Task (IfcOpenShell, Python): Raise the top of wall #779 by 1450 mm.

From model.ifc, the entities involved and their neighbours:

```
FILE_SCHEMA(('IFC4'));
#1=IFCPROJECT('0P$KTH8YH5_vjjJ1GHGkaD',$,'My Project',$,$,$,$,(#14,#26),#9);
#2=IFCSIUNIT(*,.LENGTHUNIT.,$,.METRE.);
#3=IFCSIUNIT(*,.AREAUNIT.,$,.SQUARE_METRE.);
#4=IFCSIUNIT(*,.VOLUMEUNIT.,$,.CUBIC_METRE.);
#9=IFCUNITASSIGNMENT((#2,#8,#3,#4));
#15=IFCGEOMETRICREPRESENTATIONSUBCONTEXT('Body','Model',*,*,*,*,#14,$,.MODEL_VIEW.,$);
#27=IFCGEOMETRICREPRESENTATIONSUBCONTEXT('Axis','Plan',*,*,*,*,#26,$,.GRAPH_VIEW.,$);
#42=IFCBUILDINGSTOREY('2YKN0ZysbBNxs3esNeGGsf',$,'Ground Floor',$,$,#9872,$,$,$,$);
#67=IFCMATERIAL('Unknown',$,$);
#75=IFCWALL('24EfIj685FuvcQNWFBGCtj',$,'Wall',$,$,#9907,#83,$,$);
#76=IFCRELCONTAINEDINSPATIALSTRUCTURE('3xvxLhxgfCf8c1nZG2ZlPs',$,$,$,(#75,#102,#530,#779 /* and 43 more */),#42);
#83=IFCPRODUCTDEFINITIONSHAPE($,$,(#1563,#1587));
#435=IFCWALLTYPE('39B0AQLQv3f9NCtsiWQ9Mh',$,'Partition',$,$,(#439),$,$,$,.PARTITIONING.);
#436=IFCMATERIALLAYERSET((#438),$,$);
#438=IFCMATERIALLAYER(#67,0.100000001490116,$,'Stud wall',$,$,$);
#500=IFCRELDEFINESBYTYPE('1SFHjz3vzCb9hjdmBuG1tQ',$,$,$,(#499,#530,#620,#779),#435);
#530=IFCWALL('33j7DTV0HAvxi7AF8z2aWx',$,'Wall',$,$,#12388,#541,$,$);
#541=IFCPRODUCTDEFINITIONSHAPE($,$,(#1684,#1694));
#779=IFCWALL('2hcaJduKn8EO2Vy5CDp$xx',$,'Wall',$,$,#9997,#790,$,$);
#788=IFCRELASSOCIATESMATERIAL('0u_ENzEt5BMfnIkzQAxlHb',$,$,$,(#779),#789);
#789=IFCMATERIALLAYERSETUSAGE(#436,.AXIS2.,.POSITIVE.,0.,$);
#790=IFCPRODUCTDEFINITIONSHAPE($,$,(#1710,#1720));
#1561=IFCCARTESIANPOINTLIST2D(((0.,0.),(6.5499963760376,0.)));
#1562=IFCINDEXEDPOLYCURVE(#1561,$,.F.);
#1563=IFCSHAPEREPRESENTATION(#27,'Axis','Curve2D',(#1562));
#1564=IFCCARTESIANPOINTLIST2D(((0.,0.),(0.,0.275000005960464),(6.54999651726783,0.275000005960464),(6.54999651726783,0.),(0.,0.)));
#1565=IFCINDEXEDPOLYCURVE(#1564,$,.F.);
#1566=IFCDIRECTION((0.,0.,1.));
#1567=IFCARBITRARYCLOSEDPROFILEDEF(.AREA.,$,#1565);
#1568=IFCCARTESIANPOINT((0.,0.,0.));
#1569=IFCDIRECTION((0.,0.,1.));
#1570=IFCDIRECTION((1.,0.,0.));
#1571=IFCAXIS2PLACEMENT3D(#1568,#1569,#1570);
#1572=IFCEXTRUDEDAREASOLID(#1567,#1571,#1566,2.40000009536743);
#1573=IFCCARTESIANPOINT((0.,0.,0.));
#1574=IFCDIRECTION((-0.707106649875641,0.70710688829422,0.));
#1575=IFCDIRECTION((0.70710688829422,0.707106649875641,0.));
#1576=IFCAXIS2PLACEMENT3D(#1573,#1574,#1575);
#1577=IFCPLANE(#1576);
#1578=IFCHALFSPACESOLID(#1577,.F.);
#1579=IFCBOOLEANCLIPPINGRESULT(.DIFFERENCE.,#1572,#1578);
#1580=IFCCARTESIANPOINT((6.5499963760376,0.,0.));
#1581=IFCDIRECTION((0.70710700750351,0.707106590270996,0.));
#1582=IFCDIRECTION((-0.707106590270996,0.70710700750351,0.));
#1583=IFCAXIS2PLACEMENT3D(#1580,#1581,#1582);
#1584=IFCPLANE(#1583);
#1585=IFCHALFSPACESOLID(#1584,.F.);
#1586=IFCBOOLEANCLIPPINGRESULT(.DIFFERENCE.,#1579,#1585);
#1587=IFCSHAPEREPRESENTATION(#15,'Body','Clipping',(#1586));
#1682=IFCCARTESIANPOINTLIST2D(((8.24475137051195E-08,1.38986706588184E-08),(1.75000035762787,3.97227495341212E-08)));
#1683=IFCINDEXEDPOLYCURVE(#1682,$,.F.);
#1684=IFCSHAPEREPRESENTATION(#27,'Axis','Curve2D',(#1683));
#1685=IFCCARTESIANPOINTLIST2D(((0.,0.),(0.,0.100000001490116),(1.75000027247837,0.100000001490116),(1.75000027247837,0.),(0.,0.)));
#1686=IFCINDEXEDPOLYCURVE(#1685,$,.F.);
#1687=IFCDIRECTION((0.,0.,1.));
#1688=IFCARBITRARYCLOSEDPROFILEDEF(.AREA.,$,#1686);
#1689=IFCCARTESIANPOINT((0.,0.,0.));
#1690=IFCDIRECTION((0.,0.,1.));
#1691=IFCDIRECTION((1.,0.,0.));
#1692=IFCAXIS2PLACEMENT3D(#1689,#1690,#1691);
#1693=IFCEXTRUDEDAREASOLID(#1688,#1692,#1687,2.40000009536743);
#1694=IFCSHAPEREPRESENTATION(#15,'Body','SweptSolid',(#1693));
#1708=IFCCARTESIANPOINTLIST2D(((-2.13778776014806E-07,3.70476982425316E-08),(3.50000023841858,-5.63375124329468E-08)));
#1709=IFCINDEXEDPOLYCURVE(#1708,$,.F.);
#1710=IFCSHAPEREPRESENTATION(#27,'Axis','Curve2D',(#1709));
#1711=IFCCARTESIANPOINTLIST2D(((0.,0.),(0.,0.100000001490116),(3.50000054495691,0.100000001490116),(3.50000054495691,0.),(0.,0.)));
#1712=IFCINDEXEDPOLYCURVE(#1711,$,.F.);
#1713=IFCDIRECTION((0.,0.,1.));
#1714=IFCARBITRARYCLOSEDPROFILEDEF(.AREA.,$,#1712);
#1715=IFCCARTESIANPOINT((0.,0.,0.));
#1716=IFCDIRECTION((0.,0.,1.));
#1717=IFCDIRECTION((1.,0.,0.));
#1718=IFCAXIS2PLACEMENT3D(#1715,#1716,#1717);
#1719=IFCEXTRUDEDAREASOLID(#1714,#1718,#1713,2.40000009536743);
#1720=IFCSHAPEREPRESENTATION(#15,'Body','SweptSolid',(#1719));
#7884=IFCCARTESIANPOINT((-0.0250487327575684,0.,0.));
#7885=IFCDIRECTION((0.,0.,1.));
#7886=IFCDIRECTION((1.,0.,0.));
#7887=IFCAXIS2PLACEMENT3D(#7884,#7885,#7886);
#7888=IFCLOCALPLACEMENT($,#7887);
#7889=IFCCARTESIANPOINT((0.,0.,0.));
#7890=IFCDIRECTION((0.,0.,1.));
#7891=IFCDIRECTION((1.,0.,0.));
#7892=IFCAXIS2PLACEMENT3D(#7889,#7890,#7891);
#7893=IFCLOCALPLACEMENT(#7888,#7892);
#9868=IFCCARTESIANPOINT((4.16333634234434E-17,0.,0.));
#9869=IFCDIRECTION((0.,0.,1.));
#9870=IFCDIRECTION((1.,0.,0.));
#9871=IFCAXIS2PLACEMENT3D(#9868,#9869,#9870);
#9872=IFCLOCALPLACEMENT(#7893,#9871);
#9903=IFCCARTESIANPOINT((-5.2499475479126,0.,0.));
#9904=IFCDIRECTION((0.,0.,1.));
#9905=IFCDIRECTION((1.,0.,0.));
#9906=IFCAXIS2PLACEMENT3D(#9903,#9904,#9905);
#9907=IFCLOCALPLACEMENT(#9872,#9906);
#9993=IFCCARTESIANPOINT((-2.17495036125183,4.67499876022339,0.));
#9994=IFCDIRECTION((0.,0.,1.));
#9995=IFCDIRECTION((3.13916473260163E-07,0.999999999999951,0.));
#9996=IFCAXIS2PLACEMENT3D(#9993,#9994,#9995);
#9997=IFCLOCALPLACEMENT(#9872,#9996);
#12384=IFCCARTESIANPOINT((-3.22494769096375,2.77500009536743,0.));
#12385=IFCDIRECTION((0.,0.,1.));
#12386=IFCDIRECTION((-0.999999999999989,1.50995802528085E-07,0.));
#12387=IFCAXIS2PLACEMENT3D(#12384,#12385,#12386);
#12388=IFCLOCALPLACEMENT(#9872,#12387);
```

```python
import ifcopenshell
import ifcopenshell.geom
import ifcopenshell.util.representation
import ifcopenshell.util.shape
import ifcopenshell.util.unit

model = ifcopenshell.open("model.ifc")
unit_scale = ifcopenshell.util.unit.calculate_unit_scale(model)
settings = ifcopenshell.geom.settings()


def volume(element):
    """Net volume in cubic metres, openings subtracted."""
    shape = ifcopenshell.geom.create_shape(settings, element)
    return ifcopenshell.util.shape.get_volume(shape.geometry)


wall = model.by_guid("2hcaJduKn8EO2Vy5CDp$xx")
before = volume(wall)

body = ifcopenshell.util.representation.get_representation(wall, "Model", "Body")
solid = body.Items[0]
old_height = solid.Depth
solid.Depth += 1.45 / unit_scale
after = volume(wall)

print(f"height {old_height:g} -> {solid.Depth:g}, volume {before:.3f} -> {after:.3f} m3")

model.write("model-out.ifc")
```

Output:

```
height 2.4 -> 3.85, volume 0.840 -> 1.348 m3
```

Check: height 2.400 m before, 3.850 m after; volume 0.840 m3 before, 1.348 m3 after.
